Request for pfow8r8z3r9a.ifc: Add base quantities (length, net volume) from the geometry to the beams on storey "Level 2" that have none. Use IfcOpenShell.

First a look at what the model holds.

```python
import ifcopenshell
import ifcopenshell.util.element
import ifcopenshell.util.unit

model = ifcopenshell.open("pfow8r8z3r9a.ifc")
print(model.schema)
for unit_type in ("LENGTHUNIT", "AREAUNIT", "VOLUMEUNIT"):
    print(unit_type, ifcopenshell.util.unit.calculate_unit_scale(model, unit_type))
storey = next(s for s in model.by_type("IfcBuildingStorey") if s.Name == "Level 2")
beams = [e for e in ifcopenshell.util.element.get_decomposition(storey) if e.is_a("IfcBeam")]
for e in sorted(beams, key=lambda e: e.id()):
    print(e.id(), e.is_a(), e.Name, list(ifcopenshell.util.element.get_psets(e, qtos_only=True)), sep=" | ")
```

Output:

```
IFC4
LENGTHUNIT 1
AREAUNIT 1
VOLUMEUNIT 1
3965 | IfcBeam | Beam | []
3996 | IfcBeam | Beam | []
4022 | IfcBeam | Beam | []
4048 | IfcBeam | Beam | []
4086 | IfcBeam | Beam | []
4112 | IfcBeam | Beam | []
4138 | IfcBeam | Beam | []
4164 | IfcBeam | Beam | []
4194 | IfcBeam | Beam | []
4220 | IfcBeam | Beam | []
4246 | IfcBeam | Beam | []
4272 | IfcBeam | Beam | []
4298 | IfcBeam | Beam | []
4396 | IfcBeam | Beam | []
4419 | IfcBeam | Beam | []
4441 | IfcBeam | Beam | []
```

```python
import ifcopenshell
import ifcopenshell.api.pset
import ifcopenshell.geom
import ifcopenshell.util.element
import ifcopenshell.util.shape
import ifcopenshell.util.unit

model = ifcopenshell.open("pfow8r8z3r9a.ifc")
unit_scale = ifcopenshell.util.unit.calculate_unit_scale(model)
volume_scale = ifcopenshell.util.unit.calculate_unit_scale(model, "VOLUMEUNIT")
settings = ifcopenshell.geom.settings()

storey = next(s for s in model.by_type("IfcBuildingStorey") if s.Name == "Level 2")
beams = [e for e in ifcopenshell.util.element.get_decomposition(storey) if e.is_a("IfcBeam")]

for e in sorted(beams, key=lambda e: e.id()):
    if ifcopenshell.util.element.get_psets(e, qtos_only=True, should_inherit=False):
        continue
    # Geometry comes back in metres, in the element's own axes.
    shape = ifcopenshell.geom.create_shape(settings, e)
    values = {
        "Length": ifcopenshell.util.shape.get_max_xyz(shape.geometry) / unit_scale,
        "NetVolume": ifcopenshell.util.shape.get_volume(shape.geometry) / volume_scale,
    }
    qto = ifcopenshell.api.pset.add_qto(model, product=e, name="Qto_BeamBaseQuantities")
    ifcopenshell.api.pset.edit_qto(model, qto=qto, properties=values)
    print(e.id(), {k: round(v, 3) for k, v in values.items()})

model.write("pfow8r8z3r9a_rev.ifc")
```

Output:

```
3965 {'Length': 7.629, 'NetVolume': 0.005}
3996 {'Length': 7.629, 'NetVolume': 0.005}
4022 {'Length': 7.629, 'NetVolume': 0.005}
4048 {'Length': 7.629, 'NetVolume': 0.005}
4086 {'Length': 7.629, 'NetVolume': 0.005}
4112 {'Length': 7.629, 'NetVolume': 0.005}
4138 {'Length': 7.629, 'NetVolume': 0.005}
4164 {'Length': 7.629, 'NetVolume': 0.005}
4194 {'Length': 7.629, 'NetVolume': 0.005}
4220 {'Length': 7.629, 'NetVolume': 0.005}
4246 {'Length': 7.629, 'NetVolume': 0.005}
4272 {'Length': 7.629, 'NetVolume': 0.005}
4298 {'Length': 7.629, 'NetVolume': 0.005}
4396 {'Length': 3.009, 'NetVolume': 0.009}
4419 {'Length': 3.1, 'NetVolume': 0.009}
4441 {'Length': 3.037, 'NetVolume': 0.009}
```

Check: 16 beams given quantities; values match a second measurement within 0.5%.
